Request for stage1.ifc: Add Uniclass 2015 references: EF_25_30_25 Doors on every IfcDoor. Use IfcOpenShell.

First a look at what the model holds.

```python
import ifcopenshell

model = ifcopenshell.open("stage1.ifc")
print(model.schema)
print("classifications:", [c.Name for c in model.by_type("IfcClassification")])
for ifc_class in ("IfcDoor", "IfcRoof", "IfcStair", "IfcWall", "IfcWindow"):
    print(ifc_class, len(model.by_type(ifc_class)))
```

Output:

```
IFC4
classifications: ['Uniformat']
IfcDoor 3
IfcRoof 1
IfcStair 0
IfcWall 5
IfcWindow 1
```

```python
import ifcopenshell
import ifcopenshell.api.classification

model = ifcopenshell.open("stage1.ifc")

system = ifcopenshell.api.classification.add_classification(model, classification="Uniclass 2015")

codes = {
    "IfcDoor": ("EF_25_30_25", "Doors"),
}
for ifc_class, (code, name) in codes.items():
    products = model.by_type(ifc_class)
    ifcopenshell.api.classification.add_reference(
        model, products=products, classification=system, identification=code, name=name
    )
    print(code, len(products))

model.write("stage1_rev.ifc")
```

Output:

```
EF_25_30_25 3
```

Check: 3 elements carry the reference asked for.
